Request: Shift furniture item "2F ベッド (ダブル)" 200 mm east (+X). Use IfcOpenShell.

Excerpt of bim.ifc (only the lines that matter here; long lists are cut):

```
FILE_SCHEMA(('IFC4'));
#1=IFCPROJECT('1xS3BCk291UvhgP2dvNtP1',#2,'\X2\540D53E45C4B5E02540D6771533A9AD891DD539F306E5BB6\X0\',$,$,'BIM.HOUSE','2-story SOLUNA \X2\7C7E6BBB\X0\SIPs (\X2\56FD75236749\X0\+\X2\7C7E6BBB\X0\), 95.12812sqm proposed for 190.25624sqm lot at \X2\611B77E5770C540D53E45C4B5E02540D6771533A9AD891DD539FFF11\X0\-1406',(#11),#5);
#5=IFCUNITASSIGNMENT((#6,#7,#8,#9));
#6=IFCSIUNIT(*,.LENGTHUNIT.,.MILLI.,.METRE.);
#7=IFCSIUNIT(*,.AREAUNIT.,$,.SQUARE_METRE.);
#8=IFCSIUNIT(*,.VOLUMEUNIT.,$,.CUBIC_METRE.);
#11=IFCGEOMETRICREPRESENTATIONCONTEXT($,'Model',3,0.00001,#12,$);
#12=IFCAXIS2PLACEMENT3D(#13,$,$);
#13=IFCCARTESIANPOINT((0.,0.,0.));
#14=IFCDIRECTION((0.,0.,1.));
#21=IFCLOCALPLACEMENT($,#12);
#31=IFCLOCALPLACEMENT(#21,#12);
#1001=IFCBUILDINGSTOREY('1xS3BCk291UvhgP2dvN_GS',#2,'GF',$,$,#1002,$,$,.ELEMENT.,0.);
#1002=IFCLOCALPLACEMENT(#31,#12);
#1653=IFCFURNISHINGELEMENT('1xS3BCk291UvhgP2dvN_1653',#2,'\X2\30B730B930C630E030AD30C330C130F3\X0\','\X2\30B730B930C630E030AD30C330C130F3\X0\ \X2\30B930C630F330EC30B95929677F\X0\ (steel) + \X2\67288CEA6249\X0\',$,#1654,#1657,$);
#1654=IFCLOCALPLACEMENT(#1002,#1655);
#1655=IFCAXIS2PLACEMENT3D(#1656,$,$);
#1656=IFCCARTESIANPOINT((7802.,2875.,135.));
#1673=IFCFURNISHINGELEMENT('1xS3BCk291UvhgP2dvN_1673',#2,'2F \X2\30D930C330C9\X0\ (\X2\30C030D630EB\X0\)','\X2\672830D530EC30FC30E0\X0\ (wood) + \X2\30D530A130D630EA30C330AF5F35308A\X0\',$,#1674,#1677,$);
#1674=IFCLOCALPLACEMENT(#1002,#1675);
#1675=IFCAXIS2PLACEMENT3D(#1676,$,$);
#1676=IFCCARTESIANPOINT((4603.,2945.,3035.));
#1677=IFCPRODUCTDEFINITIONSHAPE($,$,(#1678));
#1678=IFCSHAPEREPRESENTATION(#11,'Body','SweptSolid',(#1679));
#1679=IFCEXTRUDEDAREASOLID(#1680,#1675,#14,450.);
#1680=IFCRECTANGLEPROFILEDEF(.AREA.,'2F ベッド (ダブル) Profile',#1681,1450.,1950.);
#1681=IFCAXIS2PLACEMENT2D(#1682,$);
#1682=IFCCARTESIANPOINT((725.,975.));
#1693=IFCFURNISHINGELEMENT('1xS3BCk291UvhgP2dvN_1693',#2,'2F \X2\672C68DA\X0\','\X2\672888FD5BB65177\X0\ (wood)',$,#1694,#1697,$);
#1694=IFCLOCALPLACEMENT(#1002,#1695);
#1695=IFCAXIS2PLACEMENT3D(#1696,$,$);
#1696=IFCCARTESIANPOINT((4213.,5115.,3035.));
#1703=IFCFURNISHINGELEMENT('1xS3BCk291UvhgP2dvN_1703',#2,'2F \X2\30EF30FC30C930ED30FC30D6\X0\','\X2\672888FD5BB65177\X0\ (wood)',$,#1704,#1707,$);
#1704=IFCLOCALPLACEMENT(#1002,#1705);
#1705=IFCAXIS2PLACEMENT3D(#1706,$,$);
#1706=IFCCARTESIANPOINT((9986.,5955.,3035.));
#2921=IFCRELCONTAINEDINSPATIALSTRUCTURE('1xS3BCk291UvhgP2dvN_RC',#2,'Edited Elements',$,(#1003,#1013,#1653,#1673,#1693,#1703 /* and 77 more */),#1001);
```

```python
import ifcopenshell
import ifcopenshell.api.geometry
import ifcopenshell.util.placement

model = ifcopenshell.open("bim.ifc")

item = model.by_guid("1xS3BCk291UvhgP2dvN_1673")
matrix = ifcopenshell.util.placement.get_local_placement(item.ObjectPlacement)
matrix[0, 3] += 200.0
ifcopenshell.api.geometry.edit_object_placement(model, product=item, matrix=matrix, is_si=False)

print(ifcopenshell.util.placement.get_local_placement(item.ObjectPlacement).round(3) + 0.0)

model.write("bim_rev.ifc")
```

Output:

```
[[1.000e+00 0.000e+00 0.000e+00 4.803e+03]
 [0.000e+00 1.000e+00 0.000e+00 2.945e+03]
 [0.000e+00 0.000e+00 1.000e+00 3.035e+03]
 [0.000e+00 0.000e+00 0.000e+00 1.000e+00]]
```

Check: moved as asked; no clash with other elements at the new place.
